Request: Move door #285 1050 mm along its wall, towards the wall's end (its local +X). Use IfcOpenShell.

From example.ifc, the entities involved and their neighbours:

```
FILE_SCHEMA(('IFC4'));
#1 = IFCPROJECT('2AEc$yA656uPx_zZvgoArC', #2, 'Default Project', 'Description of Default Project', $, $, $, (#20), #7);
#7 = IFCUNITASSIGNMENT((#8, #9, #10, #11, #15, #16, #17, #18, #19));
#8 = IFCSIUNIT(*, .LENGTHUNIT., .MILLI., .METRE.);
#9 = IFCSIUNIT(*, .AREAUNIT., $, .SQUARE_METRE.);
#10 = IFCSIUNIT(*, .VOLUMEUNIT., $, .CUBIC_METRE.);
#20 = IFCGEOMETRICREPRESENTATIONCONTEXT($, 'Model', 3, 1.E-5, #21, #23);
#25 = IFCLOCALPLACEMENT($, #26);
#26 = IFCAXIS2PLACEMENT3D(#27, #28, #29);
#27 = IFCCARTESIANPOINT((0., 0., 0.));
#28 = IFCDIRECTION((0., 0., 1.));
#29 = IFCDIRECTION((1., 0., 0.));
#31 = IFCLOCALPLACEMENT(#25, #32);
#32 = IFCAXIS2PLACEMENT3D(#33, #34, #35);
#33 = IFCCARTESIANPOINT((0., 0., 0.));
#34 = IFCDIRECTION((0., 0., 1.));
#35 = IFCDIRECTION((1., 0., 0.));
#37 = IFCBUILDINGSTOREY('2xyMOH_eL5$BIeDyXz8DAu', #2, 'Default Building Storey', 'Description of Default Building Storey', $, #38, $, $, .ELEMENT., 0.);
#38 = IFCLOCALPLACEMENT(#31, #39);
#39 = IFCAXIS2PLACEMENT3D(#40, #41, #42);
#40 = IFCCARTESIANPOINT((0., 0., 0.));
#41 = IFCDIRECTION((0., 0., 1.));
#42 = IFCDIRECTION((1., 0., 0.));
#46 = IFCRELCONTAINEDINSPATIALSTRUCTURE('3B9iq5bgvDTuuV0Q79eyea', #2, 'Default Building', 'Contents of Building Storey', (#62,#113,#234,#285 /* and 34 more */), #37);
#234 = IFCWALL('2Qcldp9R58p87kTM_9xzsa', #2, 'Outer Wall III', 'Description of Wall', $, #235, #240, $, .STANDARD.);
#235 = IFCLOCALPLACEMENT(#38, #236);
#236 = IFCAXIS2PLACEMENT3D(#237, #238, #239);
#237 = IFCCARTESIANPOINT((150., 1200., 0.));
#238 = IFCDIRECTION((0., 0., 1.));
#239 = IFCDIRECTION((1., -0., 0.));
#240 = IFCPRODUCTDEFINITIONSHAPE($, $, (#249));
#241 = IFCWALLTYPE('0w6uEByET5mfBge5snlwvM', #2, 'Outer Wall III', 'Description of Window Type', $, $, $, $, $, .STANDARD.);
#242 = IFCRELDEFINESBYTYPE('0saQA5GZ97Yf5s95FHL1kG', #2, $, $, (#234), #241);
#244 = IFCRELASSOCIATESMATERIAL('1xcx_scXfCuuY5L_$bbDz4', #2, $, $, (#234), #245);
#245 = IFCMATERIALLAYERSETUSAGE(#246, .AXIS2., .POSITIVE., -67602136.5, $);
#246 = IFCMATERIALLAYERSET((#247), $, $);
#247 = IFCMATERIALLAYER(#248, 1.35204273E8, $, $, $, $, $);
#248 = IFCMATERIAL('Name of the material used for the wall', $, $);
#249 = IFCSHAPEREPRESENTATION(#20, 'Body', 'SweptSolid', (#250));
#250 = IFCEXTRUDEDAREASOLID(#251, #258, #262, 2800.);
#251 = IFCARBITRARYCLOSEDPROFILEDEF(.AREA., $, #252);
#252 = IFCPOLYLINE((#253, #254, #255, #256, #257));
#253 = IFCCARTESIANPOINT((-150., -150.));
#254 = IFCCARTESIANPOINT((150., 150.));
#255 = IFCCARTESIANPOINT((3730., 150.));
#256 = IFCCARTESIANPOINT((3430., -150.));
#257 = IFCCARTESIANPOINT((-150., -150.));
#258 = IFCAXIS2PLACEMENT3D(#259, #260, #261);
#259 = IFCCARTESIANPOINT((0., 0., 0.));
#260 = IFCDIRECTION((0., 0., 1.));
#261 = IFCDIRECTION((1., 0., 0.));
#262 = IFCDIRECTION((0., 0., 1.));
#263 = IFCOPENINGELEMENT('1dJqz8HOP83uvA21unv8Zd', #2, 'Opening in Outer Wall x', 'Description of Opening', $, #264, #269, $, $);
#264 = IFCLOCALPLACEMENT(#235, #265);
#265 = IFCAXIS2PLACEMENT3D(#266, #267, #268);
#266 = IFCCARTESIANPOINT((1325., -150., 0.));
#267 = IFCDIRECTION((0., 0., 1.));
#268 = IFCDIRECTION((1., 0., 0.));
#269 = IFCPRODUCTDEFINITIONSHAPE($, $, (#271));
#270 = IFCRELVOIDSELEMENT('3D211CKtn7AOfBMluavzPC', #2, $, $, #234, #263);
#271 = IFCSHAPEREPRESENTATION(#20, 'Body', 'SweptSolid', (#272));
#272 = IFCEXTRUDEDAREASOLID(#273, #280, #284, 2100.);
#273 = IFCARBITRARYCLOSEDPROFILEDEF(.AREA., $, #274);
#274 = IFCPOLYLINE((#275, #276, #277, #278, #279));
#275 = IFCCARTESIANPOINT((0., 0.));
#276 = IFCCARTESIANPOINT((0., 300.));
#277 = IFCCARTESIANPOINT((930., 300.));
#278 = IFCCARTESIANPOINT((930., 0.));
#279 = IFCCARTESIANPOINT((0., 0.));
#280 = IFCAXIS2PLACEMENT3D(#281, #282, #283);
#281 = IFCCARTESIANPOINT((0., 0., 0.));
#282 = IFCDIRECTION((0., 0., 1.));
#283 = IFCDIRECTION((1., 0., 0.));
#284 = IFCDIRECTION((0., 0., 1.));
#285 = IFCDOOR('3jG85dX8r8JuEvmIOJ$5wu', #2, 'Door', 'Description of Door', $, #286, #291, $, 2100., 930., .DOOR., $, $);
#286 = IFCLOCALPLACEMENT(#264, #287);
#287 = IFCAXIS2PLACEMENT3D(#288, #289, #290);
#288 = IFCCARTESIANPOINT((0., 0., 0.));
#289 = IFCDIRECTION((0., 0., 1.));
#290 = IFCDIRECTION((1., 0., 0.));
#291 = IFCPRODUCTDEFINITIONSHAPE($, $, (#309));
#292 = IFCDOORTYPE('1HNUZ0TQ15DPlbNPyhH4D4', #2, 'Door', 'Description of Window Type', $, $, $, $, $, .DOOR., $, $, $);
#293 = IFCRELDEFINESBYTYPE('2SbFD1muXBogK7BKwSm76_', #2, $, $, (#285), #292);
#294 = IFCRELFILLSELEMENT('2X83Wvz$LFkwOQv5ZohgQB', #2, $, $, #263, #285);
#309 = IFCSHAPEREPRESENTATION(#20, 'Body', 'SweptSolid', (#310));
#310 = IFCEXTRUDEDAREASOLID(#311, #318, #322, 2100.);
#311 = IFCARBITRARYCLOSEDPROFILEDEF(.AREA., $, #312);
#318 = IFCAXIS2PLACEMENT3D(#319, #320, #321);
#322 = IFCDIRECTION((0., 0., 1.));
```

```python
import ifcopenshell
import ifcopenshell.api.geometry
import ifcopenshell.util.placement

model = ifcopenshell.open("example.ifc")

door = model.by_guid("3jG85dX8r8JuEvmIOJ$5wu")
opening = door.FillsVoids[0].RelatingOpeningElement
wall = opening.VoidsElements[0].RelatingBuildingElement

wall_matrix = ifcopenshell.util.placement.get_local_placement(wall.ObjectPlacement)
shift = wall_matrix[:3, 0] * 1050.0
before = ifcopenshell.util.placement.get_local_placement(door.ObjectPlacement)[:3, 3].copy()

# The door is placed relative to its opening, so it follows when the opening moves.
matrix = ifcopenshell.util.placement.get_local_placement(opening.ObjectPlacement)
matrix[:3, 3] += shift
ifcopenshell.api.geometry.edit_object_placement(
    model, product=opening, matrix=matrix, is_si=False, should_transform_children=True
)

after = ifcopenshell.util.placement.get_local_placement(door.ObjectPlacement)[:3, 3]
print("door moved by", (after - before).round(3) + 0.0)

model.write("example_v2.ifc")
```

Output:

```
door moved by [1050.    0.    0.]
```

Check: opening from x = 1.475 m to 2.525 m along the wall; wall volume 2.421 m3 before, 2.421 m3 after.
